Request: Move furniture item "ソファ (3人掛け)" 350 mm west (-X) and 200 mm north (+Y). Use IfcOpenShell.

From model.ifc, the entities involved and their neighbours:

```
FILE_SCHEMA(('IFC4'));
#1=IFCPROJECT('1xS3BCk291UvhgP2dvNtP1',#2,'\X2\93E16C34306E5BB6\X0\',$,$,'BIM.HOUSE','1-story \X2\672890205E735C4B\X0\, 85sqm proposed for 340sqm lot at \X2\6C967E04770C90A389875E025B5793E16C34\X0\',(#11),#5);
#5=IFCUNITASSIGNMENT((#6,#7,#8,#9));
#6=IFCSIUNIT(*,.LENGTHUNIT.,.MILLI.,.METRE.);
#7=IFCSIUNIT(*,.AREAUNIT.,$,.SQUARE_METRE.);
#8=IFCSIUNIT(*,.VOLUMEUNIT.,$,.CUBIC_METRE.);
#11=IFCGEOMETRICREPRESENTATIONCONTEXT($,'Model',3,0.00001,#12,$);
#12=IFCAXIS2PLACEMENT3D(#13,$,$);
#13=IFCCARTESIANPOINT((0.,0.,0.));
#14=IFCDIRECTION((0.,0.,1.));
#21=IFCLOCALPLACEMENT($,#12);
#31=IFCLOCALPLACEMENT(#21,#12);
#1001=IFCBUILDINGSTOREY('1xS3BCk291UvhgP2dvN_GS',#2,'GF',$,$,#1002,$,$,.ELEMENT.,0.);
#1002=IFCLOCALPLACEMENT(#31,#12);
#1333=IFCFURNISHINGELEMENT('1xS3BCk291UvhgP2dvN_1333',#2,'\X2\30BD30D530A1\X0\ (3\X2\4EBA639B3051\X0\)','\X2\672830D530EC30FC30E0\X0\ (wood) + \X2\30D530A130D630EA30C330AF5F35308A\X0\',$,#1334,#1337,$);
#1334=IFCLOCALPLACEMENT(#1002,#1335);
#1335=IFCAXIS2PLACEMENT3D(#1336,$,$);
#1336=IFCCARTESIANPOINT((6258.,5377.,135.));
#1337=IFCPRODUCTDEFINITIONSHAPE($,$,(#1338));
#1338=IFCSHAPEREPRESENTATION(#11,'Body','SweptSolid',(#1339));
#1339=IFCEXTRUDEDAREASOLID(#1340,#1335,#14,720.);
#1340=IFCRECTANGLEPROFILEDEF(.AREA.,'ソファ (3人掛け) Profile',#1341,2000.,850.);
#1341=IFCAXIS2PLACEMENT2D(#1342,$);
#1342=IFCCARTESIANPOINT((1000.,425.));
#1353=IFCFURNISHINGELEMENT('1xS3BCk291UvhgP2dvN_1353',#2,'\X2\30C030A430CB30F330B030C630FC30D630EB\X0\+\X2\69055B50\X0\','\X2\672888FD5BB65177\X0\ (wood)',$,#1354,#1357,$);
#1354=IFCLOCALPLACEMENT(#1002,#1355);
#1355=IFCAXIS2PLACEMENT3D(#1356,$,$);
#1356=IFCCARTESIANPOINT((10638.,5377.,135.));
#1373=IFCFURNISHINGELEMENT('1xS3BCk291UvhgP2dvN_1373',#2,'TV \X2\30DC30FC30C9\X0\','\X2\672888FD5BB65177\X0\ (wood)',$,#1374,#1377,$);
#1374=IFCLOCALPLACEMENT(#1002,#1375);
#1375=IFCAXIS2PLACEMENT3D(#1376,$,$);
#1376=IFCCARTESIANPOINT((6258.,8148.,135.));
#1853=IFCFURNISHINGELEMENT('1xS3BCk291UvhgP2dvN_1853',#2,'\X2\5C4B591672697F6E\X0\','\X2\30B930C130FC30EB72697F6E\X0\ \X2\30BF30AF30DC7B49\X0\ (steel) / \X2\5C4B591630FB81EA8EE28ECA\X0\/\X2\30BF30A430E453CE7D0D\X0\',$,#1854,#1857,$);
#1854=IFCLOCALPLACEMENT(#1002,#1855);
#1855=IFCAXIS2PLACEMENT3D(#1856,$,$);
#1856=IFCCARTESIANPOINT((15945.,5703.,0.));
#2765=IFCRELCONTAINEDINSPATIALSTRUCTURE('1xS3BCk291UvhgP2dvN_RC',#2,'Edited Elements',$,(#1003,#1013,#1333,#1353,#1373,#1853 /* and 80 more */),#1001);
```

```python
import ifcopenshell
import ifcopenshell.api.geometry
import ifcopenshell.util.placement

model = ifcopenshell.open("model.ifc")

item = model.by_guid("1xS3BCk291UvhgP2dvN_1333")
matrix = ifcopenshell.util.placement.get_local_placement(item.ObjectPlacement)
matrix[0, 3] -= 350.0
matrix[1, 3] += 200.0
ifcopenshell.api.geometry.edit_object_placement(model, product=item, matrix=matrix, is_si=False)

print(ifcopenshell.util.placement.get_local_placement(item.ObjectPlacement).round(3) + 0.0)

model.write("model_updated.ifc")
```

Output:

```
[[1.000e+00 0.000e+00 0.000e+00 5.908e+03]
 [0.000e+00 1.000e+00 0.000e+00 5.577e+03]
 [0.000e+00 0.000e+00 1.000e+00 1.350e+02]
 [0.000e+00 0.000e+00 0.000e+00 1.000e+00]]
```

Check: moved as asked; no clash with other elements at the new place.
